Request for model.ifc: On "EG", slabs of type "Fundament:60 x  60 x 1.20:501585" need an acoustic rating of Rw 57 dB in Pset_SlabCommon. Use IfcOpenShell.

First a look at what the model holds.

```python
import ifcopenshell
import ifcopenshell.util.element

model = ifcopenshell.open("model.ifc")
print(model.schema)
storey = next(s for s in model.by_type("IfcBuildingStorey") if s.Name == "EG")
slabs = [e for e in ifcopenshell.util.element.get_decomposition(storey) if e.is_a("IfcSlab")]
seen = {}
for e in slabs:
    element_type = ifcopenshell.util.element.get_type(e)
    key = (element_type.Name if element_type != e and element_type else None, ifcopenshell.util.element.get_pset(e, "Pset_SlabCommon", "AcousticRating"))
    seen[key] = seen.get(key, 0) + 1
for (name, value), count in sorted(seen.items(), key=str):
    print(count, "x", name, "|", value)
```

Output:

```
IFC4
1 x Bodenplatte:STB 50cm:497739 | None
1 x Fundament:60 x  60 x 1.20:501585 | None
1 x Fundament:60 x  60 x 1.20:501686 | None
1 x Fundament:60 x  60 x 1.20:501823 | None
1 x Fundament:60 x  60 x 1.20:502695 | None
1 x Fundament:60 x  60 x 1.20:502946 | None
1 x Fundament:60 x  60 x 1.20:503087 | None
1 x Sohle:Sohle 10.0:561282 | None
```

```python
import ifcopenshell
import ifcopenshell.api.pset
import ifcopenshell.util.element

model = ifcopenshell.open("model.ifc")

storey = next(s for s in model.by_type("IfcBuildingStorey") if s.Name == "EG")
slabs = [e for e in ifcopenshell.util.element.get_decomposition(storey) if e.is_a("IfcSlab")]

count = 0
for e in slabs:
    element_type = ifcopenshell.util.element.get_type(e)
    if element_type in (None, e) or element_type.Name != "Fundament:60 x  60 x 1.20:501585":
        continue
    # add_pset returns the element's existing set when there is one.
    pset = ifcopenshell.api.pset.add_pset(model, product=e, name="Pset_SlabCommon")
    ifcopenshell.api.pset.edit_pset(model, pset=pset, properties={"AcousticRating": "Rw 57 dB"})
    count += 1

print(count, "slabs updated")

model.write("model_v2.ifc")
```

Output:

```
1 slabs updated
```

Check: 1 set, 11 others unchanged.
